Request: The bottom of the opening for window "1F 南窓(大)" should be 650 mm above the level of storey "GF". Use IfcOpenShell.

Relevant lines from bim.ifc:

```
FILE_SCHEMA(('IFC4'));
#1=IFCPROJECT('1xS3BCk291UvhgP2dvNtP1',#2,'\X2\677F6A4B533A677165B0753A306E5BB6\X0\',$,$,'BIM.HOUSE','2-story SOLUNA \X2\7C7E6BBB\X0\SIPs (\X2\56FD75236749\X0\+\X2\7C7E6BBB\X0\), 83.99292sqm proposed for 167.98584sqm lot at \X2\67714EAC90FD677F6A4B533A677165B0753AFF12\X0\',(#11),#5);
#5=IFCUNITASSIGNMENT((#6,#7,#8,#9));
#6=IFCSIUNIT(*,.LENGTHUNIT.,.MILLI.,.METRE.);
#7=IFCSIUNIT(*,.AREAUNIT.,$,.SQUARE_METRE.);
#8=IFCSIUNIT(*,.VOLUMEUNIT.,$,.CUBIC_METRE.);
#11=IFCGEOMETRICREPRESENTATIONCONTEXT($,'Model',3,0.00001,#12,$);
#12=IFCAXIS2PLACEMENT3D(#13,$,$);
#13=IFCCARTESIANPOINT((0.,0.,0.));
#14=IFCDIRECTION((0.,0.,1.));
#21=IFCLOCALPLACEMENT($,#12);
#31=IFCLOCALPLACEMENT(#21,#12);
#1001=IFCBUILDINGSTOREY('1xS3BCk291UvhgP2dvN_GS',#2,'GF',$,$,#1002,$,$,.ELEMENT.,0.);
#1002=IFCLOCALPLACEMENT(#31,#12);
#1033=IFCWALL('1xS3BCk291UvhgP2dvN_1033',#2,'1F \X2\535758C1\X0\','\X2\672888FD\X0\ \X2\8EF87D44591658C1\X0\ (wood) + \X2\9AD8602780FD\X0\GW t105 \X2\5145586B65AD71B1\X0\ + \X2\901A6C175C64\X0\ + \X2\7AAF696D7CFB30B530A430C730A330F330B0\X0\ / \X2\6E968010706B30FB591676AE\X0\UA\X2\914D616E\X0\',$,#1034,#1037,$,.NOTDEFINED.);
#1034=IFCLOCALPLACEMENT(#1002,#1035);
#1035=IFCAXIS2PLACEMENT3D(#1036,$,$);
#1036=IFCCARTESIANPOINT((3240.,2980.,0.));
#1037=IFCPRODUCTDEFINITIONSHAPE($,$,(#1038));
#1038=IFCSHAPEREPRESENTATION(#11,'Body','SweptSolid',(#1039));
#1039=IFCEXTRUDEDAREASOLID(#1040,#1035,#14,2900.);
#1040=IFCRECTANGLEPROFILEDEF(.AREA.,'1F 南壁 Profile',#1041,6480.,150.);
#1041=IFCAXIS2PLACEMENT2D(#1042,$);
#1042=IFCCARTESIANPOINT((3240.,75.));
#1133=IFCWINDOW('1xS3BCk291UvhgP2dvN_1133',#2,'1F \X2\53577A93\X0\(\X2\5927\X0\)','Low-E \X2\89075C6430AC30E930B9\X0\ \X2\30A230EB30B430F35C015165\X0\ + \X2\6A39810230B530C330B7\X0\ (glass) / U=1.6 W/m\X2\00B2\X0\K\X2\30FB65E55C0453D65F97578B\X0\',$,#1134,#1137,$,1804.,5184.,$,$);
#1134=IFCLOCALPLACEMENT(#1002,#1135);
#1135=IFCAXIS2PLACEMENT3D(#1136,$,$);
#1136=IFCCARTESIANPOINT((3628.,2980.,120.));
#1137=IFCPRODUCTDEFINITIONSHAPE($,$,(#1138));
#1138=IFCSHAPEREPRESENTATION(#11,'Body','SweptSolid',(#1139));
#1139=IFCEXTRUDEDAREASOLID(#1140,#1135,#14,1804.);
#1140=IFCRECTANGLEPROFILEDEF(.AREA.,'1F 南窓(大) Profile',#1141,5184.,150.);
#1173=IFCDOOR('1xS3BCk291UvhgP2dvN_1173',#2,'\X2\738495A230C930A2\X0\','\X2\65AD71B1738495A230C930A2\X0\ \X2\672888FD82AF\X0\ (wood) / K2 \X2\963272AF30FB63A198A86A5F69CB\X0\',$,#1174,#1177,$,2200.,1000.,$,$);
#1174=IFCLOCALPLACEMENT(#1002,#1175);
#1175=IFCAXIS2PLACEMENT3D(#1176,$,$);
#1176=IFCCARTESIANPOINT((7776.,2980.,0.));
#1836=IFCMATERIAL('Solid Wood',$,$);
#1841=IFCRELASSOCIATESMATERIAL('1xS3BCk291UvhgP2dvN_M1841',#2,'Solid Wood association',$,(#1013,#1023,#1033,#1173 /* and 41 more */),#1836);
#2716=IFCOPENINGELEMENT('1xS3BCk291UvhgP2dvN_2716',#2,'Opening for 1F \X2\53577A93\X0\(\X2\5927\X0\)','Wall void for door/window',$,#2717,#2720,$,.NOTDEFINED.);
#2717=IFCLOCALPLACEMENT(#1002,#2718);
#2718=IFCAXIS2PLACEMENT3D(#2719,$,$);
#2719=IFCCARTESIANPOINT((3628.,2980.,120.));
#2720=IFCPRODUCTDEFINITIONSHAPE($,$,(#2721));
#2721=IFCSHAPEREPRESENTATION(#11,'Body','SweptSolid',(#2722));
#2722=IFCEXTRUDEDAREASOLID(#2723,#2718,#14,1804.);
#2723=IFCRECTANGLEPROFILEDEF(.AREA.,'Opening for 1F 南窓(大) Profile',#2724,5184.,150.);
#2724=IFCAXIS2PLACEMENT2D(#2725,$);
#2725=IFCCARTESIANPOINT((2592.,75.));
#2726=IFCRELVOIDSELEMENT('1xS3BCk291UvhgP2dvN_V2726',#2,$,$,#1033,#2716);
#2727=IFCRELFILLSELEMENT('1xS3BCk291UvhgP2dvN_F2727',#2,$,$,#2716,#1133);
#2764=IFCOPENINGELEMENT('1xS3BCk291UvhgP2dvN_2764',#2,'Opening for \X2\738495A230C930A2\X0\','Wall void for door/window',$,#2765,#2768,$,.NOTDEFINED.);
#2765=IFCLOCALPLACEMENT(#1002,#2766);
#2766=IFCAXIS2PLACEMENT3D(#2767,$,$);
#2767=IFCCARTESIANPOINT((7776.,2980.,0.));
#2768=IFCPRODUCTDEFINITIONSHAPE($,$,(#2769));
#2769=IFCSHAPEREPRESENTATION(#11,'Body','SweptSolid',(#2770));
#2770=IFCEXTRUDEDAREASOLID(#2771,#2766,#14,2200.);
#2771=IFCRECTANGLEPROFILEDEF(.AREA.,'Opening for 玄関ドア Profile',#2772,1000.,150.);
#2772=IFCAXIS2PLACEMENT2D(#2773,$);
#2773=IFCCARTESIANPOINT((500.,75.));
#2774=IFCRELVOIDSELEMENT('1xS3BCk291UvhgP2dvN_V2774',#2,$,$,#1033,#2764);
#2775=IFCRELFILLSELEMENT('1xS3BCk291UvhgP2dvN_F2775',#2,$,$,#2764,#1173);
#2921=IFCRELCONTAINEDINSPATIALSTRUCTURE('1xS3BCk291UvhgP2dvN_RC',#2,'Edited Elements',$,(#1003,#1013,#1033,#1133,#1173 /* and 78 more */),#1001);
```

```python
import numpy as np
import ifcopenshell
import ifcopenshell.api.geometry
import ifcopenshell.geom
import ifcopenshell.util.element
import ifcopenshell.util.placement
import ifcopenshell.util.shape
import ifcopenshell.util.unit

model = ifcopenshell.open("bim.ifc")
unit_scale = ifcopenshell.util.unit.calculate_unit_scale(model)

window = model.by_guid("1xS3BCk291UvhgP2dvN_1133")
opening = window.FillsVoids[0].RelatingOpeningElement
storey = ifcopenshell.util.element.get_container(window, ifc_class="IfcBuildingStorey")
level = ifcopenshell.util.placement.get_local_placement(storey.ObjectPlacement)[2, 3]

# The opening's origin need not be at the sill, so measure its lowest point.
shape = ifcopenshell.geom.create_shape(ifcopenshell.geom.settings(), opening)
bottom = ifcopenshell.util.shape.get_shape_bottom_elevation(shape, shape.geometry) / unit_scale
dz = level + 0.65 / unit_scale - bottom

shift = np.array([0.0, 0.0, dz])
# The window is not placed relative to its opening, so move both.
for product in (opening, window):
    matrix = ifcopenshell.util.placement.get_local_placement(product.ObjectPlacement)
    matrix[:3, 3] += shift
    ifcopenshell.api.geometry.edit_object_placement(model, product=product, matrix=matrix, is_si=False)

print(f"moved by {dz * unit_scale:+.3f} m")

model.write("bim_edited.ifc")
```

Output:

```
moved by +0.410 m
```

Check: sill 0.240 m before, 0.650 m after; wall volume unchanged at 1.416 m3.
